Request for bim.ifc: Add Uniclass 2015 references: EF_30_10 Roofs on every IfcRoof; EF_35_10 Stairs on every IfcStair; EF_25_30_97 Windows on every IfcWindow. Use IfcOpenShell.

First a look at what the model holds.

```python
import ifcopenshell

model = ifcopenshell.open("bim.ifc")
print(model.schema)
print("classifications:", [c.Name for c in model.by_type("IfcClassification")])
for ifc_class in ("IfcDoor", "IfcRoof", "IfcStair", "IfcWall", "IfcWindow"):
    print(ifc_class, len(model.by_type(ifc_class)))
```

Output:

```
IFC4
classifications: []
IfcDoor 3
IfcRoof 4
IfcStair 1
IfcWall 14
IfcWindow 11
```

```python
import ifcopenshell
import ifcopenshell.api.classification

model = ifcopenshell.open("bim.ifc")

system = ifcopenshell.api.classification.add_classification(model, classification="Uniclass 2015")

codes = {
    "IfcRoof": ("EF_30_10", "Roofs"),
    "IfcStair": ("EF_35_10", "Stairs"),
    "IfcWindow": ("EF_25_30_97", "Windows"),
}
for ifc_class, (code, name) in codes.items():
    products = model.by_type(ifc_class)
    ifcopenshell.api.classification.add_reference(
        model, products=products, classification=system, identification=code, name=name
    )
    print(code, len(products))

model.write("bim_rev.ifc")
```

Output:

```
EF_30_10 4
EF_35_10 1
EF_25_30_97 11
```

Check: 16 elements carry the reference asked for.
